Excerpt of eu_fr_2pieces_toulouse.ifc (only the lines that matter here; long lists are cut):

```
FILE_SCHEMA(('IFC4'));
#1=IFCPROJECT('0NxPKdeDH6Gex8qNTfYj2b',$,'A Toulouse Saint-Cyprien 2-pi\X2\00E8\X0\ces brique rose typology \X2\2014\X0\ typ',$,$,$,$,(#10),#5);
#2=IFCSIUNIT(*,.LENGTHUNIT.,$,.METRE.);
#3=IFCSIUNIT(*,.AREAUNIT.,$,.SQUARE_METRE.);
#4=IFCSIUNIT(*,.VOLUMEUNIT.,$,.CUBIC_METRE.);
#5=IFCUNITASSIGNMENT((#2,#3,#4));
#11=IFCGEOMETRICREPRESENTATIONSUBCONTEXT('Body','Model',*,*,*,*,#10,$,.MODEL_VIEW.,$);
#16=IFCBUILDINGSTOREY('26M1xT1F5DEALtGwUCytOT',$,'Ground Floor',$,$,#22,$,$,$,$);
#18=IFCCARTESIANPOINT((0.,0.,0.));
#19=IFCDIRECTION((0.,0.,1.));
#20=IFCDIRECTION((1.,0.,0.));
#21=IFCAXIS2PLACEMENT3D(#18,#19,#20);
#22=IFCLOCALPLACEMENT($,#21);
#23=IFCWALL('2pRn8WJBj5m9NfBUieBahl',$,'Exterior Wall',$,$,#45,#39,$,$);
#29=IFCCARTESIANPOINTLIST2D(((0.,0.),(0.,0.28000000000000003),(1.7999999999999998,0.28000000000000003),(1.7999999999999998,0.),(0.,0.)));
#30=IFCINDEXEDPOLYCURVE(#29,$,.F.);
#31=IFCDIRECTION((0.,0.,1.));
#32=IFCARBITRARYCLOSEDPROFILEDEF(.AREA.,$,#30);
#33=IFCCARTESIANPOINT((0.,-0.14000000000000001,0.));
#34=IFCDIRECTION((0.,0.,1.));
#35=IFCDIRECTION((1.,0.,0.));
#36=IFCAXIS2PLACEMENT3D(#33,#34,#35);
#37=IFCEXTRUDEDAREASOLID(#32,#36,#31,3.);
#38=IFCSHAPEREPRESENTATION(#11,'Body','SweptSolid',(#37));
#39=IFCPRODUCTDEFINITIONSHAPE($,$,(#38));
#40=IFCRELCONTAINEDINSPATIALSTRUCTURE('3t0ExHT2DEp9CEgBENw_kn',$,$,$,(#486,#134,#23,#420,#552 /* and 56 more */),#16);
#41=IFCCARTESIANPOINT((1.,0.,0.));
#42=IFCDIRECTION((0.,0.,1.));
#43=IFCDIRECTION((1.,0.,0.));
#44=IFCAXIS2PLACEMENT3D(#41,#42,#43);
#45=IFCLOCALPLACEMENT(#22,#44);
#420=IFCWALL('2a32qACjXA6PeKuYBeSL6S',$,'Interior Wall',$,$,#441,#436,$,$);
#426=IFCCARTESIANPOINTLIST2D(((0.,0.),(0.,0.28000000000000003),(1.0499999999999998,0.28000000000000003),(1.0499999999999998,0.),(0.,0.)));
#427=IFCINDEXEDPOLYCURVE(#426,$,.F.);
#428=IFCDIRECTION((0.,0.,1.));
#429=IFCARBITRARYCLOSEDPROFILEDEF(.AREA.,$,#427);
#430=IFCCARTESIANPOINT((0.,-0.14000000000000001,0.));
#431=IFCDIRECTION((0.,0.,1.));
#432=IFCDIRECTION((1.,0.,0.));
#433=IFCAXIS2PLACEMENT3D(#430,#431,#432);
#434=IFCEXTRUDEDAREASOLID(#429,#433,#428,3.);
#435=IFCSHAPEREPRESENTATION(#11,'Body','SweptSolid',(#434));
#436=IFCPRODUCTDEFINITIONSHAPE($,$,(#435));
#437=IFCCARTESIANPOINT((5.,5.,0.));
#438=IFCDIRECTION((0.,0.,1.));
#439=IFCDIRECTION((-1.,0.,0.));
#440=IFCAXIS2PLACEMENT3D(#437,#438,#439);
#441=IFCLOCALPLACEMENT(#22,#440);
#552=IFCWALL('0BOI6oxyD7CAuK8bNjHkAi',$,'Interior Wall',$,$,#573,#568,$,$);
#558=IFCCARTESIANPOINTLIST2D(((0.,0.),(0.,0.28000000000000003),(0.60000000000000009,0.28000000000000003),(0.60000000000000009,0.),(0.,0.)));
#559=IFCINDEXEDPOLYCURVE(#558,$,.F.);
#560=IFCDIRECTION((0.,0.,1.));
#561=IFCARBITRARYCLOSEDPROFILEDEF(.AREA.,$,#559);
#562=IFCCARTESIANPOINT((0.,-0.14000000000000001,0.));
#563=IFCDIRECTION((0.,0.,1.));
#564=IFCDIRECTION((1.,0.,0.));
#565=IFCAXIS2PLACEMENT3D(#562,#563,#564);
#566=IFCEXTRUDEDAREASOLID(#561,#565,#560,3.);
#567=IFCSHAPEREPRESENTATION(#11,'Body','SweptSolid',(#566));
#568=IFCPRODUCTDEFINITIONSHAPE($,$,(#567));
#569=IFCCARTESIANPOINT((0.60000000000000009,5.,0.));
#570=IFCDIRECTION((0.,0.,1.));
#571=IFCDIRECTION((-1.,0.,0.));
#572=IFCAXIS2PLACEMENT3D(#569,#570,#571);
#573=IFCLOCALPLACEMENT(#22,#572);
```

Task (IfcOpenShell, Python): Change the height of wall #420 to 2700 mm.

```python
import ifcopenshell
import ifcopenshell.geom
import ifcopenshell.util.representation
import ifcopenshell.util.shape

model = ifcopenshell.open("eu_fr_2pieces_toulouse.ifc")
settings = ifcopenshell.geom.settings()


def volume(element):
    """Net volume in cubic metres, openings subtracted."""
    shape = ifcopenshell.geom.create_shape(settings, element)
    return ifcopenshell.util.shape.get_volume(shape.geometry)


wall = model.by_id(420)
before = volume(wall)

body = ifcopenshell.util.representation.get_representation(wall, "Model", "Body")
solid = body.Items[0]
old_height = solid.Depth
solid.Depth = 2.7
after = volume(wall)

print(f"height {old_height:g} -> {solid.Depth:g}, volume {before:.3f} -> {after:.3f} m3")

model.write("eu_fr_2pieces_toulouse-out.ifc")
```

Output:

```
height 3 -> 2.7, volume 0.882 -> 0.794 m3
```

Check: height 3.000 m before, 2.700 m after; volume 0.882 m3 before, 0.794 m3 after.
